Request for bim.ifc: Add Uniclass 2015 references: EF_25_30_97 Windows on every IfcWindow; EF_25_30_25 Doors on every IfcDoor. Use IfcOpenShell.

First a look at what the model holds.

```python
import ifcopenshell

model = ifcopenshell.open("bim.ifc")
print(model.schema)
print("classifications:", [c.Name for c in model.by_type("IfcClassification")])
for ifc_class in ("IfcDoor", "IfcRoof", "IfcStair", "IfcWall", "IfcWindow"):
    print(ifc_class, len(model.by_type(ifc_class)))
```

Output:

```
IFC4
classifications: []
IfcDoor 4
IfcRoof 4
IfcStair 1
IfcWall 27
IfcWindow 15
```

```python
import ifcopenshell
import ifcopenshell.api.classification

model = ifcopenshell.open("bim.ifc")

system = ifcopenshell.api.classification.add_classification(model, classification="Uniclass 2015")

codes = {
    "IfcWindow": ("EF_25_30_97", "Windows"),
    "IfcDoor": ("EF_25_30_25", "Doors"),
}
for ifc_class, (code, name) in codes.items():
    products = model.by_type(ifc_class)
    ifcopenshell.api.classification.add_reference(
        model, products=products, classification=system, identification=code, name=name
    )
    print(code, len(products))

model.write("bim_edited.ifc")
```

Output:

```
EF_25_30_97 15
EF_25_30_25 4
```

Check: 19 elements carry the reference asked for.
